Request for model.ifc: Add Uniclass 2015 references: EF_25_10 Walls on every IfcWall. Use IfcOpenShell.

First a look at what the model holds.

```python
import ifcopenshell

model = ifcopenshell.open("model.ifc")
print(model.schema)
print("classifications:", [c.Name for c in model.by_type("IfcClassification")])
for ifc_class in ("IfcDoor", "IfcRoof", "IfcStair", "IfcWall", "IfcWindow"):
    print(ifc_class, len(model.by_type(ifc_class)))
```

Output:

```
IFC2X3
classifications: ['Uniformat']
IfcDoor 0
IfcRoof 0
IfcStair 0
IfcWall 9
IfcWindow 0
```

```python
import ifcopenshell
import ifcopenshell.api.classification

model = ifcopenshell.open("model.ifc")

# IFC2X3 requires Source and Edition and has no link from the project to the system.
system = model.create_entity("IfcClassification", Source="NBS", Edition="2015", Name="Uniclass 2015")

codes = {
    "IfcWall": ("EF_25_10", "Walls"),
}
for ifc_class, (code, name) in codes.items():
    products = model.by_type(ifc_class)
    ifcopenshell.api.classification.add_reference(
        model, products=products, classification=system, identification=code, name=name
    )
    print(code, len(products))

model.write("model_edited.ifc")
```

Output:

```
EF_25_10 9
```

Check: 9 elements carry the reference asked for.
